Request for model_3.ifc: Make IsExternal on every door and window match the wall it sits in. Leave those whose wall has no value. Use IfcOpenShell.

First a look at what the model holds.

```python
import ifcopenshell
import ifcopenshell.util.element

model = ifcopenshell.open("model_3.ifc")
print(model.schema)
seen = {}
for e in model.by_type("IfcDoor") + model.by_type("IfcWindow"):
    if not e.FillsVoids:
        continue
    host = e.FillsVoids[0].RelatingOpeningElement.VoidsElements[0].RelatingBuildingElement
    own = ifcopenshell.util.element.get_pset(e, f"Pset_{e.is_a()[3:].removesuffix('StandardCase')}Common", "IsExternal")
    wall = ifcopenshell.util.element.get_pset(host, "Pset_WallCommon", "IsExternal")
    seen[e.is_a(), own, wall] = seen.get((e.is_a(), own, wall), 0) + 1
for (cls, own, wall), count in sorted(seen.items(), key=str):
    print(count, cls, "IsExternal:", own, "| host wall:", wall)
```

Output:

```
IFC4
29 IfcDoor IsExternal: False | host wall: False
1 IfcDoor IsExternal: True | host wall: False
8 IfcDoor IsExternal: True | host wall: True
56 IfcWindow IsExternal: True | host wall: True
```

```python
import ifcopenshell
import ifcopenshell.api.pset
import ifcopenshell.util.element

model = ifcopenshell.open("model_3.ifc")

count = 0
for ifc_class, pset_name in (("IfcDoor", "Pset_DoorCommon"), ("IfcWindow", "Pset_WindowCommon")):
    for e in model.by_type(ifc_class):
        if not e.FillsVoids:
            continue
        host = e.FillsVoids[0].RelatingOpeningElement.VoidsElements[0].RelatingBuildingElement
        external = ifcopenshell.util.element.get_pset(host, "Pset_WallCommon", "IsExternal")
        if external is None or ifcopenshell.util.element.get_pset(e, pset_name, "IsExternal") == external:
            continue
        pset = ifcopenshell.api.pset.add_pset(model, product=e, name=pset_name)
        ifcopenshell.api.pset.edit_pset(model, pset=pset, properties={"IsExternal": external})
        count += 1

print(count, "updated")

model.write("model_3_rev.ifc")
```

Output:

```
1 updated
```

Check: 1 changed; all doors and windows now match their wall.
